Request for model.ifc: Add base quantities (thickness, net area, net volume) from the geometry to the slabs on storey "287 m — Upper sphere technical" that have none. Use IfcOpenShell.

First a look at what the model holds.

```python
import ifcopenshell
import ifcopenshell.util.element
import ifcopenshell.util.unit

model = ifcopenshell.open("model.ifc")
print(model.schema)
for unit_type in ("LENGTHUNIT", "AREAUNIT", "VOLUMEUNIT"):
    print(unit_type, ifcopenshell.util.unit.calculate_unit_scale(model, unit_type))
storey = next(s for s in model.by_type("IfcBuildingStorey") if s.Name == "287 m — Upper sphere technical")
slabs = [e for e in ifcopenshell.util.element.get_decomposition(storey) if e.is_a("IfcSlab")]
for e in sorted(slabs, key=lambda e: e.id()):
    print(e.id(), e.is_a(), e.Name, list(ifcopenshell.util.element.get_psets(e, qtos_only=True)), sep=" | ")
```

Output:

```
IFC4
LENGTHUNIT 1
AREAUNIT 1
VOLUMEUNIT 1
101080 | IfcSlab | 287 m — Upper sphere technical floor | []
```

```python
import ifcopenshell
import ifcopenshell.api.pset
import ifcopenshell.geom
import ifcopenshell.util.element
import ifcopenshell.util.shape
import ifcopenshell.util.unit

model = ifcopenshell.open("model.ifc")
unit_scale = ifcopenshell.util.unit.calculate_unit_scale(model)
area_scale = ifcopenshell.util.unit.calculate_unit_scale(model, "AREAUNIT")
volume_scale = ifcopenshell.util.unit.calculate_unit_scale(model, "VOLUMEUNIT")
settings = ifcopenshell.geom.settings()

storey = next(s for s in model.by_type("IfcBuildingStorey") if s.Name == "287 m — Upper sphere technical")
slabs = [e for e in ifcopenshell.util.element.get_decomposition(storey) if e.is_a("IfcSlab")]

for e in sorted(slabs, key=lambda e: e.id()):
    if ifcopenshell.util.element.get_psets(e, qtos_only=True, should_inherit=False):
        continue
    # Geometry comes back in metres, in the element's own axes.
    shape = ifcopenshell.geom.create_shape(settings, e)
    values = {
        "Width": ifcopenshell.util.shape.get_z(shape.geometry) / unit_scale,
        "NetArea": ifcopenshell.util.shape.get_footprint_area(shape.geometry) / area_scale,
        "NetVolume": ifcopenshell.util.shape.get_volume(shape.geometry) / volume_scale,
    }
    qto = ifcopenshell.api.pset.add_qto(model, product=e, name="Qto_SlabBaseQuantities")
    ifcopenshell.api.pset.edit_qto(model, qto=qto, properties=values)
    print(e.id(), {k: round(v, 3) for k, v in values.items()})

model.write("model_v2.ifc")
```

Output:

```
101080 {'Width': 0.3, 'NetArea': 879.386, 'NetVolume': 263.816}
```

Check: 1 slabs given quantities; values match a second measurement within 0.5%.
